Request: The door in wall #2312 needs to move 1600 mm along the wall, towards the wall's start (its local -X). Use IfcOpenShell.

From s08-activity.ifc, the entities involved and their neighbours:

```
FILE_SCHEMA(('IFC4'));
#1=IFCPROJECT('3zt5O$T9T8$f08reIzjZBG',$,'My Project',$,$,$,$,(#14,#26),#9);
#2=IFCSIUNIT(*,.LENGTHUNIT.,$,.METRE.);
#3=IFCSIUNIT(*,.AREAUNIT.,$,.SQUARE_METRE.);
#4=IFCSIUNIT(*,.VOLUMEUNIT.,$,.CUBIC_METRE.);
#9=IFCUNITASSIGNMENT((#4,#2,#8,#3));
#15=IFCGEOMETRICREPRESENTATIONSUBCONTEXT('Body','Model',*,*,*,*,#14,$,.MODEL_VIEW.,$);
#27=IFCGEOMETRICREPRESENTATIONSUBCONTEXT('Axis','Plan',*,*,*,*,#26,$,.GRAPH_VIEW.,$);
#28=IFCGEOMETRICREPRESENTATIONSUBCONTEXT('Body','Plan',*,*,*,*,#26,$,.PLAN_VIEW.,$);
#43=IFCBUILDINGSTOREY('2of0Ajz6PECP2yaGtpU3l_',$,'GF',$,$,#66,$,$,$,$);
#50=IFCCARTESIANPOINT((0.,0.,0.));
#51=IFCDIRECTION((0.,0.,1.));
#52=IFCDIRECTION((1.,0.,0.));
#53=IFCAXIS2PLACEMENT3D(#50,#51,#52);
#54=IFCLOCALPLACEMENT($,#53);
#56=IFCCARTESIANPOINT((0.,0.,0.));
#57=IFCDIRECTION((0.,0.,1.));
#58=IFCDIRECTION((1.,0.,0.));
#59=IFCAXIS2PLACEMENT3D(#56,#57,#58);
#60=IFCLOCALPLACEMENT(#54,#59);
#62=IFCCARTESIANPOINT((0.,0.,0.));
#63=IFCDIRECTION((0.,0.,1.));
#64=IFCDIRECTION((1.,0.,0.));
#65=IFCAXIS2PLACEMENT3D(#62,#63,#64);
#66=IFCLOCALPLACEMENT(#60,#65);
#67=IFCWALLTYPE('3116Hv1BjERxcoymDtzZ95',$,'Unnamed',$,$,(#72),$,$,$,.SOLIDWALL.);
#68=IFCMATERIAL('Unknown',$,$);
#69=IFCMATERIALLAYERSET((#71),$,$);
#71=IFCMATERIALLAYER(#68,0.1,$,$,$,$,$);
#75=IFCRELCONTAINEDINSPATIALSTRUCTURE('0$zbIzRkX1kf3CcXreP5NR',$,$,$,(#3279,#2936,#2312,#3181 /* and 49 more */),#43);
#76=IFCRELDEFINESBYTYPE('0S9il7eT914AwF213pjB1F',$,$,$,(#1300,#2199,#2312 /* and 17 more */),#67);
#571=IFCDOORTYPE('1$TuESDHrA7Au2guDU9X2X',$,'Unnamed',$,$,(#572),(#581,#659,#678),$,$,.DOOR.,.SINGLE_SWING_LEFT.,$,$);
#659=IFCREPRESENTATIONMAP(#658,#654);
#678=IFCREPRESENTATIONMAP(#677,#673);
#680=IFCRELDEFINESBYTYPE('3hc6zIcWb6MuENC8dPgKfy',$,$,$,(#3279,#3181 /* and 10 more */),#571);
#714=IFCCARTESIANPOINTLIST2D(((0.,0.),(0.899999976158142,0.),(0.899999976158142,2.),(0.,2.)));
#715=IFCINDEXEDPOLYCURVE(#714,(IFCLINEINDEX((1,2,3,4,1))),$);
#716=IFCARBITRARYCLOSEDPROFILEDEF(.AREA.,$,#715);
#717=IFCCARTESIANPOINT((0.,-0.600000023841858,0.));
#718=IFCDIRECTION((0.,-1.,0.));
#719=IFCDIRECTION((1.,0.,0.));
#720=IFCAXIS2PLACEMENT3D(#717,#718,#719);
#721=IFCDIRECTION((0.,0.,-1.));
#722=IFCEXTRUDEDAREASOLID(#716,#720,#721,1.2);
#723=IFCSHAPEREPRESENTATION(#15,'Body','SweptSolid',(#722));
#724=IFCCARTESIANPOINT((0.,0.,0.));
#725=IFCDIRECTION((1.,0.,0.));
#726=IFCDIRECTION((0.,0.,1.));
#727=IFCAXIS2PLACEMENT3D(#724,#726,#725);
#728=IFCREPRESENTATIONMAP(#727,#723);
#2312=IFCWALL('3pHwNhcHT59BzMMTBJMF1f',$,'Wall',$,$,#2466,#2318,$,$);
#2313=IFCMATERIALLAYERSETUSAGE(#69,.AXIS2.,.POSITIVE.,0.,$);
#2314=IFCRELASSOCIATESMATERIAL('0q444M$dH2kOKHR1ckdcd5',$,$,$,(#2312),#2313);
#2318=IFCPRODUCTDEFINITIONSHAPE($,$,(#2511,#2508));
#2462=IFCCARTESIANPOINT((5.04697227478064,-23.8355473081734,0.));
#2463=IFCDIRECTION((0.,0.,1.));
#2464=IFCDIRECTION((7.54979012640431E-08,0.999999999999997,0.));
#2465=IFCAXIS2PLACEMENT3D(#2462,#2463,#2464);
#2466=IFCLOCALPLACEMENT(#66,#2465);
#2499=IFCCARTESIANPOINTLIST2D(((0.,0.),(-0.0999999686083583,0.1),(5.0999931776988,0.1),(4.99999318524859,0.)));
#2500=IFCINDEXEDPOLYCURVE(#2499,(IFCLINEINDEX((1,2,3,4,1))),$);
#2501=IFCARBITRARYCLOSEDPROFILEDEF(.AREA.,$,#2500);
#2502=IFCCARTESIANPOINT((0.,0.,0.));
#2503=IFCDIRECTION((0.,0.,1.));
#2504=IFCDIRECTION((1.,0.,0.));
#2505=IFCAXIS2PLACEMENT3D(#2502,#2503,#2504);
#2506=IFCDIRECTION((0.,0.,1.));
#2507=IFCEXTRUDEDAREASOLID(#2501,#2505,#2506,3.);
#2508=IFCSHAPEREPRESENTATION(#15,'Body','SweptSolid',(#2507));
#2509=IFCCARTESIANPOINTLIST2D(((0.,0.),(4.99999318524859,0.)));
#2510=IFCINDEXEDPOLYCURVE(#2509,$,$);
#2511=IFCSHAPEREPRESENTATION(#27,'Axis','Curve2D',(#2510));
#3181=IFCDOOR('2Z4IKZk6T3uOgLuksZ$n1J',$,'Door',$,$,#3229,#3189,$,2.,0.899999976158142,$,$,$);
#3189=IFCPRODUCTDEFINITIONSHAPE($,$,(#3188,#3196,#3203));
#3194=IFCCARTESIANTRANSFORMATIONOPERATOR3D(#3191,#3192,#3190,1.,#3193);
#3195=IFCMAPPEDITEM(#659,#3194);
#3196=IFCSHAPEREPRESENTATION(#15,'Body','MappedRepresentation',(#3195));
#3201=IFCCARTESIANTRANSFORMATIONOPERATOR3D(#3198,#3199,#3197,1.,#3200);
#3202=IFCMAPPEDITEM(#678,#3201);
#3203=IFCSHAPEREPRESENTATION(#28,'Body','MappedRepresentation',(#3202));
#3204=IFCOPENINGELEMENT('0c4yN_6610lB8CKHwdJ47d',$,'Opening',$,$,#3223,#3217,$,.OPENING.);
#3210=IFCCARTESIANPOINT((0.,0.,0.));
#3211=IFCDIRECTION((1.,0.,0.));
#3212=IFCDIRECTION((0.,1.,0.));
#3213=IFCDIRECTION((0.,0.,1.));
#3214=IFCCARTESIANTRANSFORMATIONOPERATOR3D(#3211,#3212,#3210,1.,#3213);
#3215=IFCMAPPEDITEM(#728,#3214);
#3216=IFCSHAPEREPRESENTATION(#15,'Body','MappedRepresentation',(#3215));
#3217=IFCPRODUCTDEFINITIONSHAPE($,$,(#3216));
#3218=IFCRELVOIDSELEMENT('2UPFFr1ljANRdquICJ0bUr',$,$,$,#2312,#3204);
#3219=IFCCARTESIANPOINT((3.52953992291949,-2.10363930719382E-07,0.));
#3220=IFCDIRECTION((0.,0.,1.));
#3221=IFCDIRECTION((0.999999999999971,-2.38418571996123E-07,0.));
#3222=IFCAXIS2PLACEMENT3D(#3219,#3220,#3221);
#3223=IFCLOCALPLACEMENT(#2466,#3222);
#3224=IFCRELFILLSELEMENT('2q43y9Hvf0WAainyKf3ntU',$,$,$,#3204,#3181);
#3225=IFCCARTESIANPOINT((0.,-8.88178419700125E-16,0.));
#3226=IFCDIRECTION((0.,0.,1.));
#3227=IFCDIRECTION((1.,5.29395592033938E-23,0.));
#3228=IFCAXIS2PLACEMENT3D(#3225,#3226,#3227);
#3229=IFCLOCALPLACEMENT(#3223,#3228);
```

```python
import ifcopenshell
import ifcopenshell.api.geometry
import ifcopenshell.util.placement
import ifcopenshell.util.unit

model = ifcopenshell.open("s08-activity.ifc")
unit_scale = ifcopenshell.util.unit.calculate_unit_scale(model)

door = model.by_guid("2Z4IKZk6T3uOgLuksZ$n1J")
opening = door.FillsVoids[0].RelatingOpeningElement
wall = opening.VoidsElements[0].RelatingBuildingElement

wall_matrix = ifcopenshell.util.placement.get_local_placement(wall.ObjectPlacement)
shift = wall_matrix[:3, 0] * -1.6 / unit_scale
before = ifcopenshell.util.placement.get_local_placement(door.ObjectPlacement)[:3, 3].copy()

# The door is placed relative to its opening, so it follows when the opening moves.
matrix = ifcopenshell.util.placement.get_local_placement(opening.ObjectPlacement)
matrix[:3, 3] += shift
ifcopenshell.api.geometry.edit_object_placement(
    model, product=opening, matrix=matrix, is_si=False, should_transform_children=True
)

after = ifcopenshell.util.placement.get_local_placement(door.ObjectPlacement)[:3, 3]
print("door moved by", (after - before).round(3) + 0.0)

model.write("s08-activity-out.ifc")
```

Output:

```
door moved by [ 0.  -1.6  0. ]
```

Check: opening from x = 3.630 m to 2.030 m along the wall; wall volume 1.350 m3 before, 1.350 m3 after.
